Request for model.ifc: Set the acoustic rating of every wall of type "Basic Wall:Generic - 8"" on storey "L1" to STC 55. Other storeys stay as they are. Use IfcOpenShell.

First a look at what the model holds.

```python
import ifcopenshell
import ifcopenshell.util.element

model = ifcopenshell.open("model.ifc")
print(model.schema)
storey = next(s for s in model.by_type("IfcBuildingStorey") if s.Name == "L1")
walls = [e for e in ifcopenshell.util.element.get_decomposition(storey) if e.is_a("IfcWall")]
seen = {}
for e in walls:
    element_type = ifcopenshell.util.element.get_type(e)
    key = (element_type.Name if element_type != e and element_type else None, ifcopenshell.util.element.get_pset(e, "Pset_WallCommon", "AcousticRating"))
    seen[key] = seen.get(key, 0) + 1
for (name, value), count in sorted(seen.items(), key=str):
    print(count, "x", name, "|", value)
```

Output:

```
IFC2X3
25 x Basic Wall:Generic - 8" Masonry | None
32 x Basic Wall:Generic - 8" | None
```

```python
import ifcopenshell
import ifcopenshell.api.pset
import ifcopenshell.util.element

model = ifcopenshell.open("model.ifc")

storey = next(s for s in model.by_type("IfcBuildingStorey") if s.Name == "L1")
walls = [e for e in ifcopenshell.util.element.get_decomposition(storey) if e.is_a("IfcWall")]

count = 0
for e in walls:
    element_type = ifcopenshell.util.element.get_type(e)
    if element_type in (None, e) or element_type.Name != 'Basic Wall:Generic - 8"':
        continue
    # add_pset returns the element's existing set when there is one.
    pset = ifcopenshell.api.pset.add_pset(model, product=e, name="Pset_WallCommon")
    ifcopenshell.api.pset.edit_pset(model, pset=pset, properties={"AcousticRating": "STC 55"})
    count += 1

print(count, "walls updated")

model.write("model_v2.ifc")
```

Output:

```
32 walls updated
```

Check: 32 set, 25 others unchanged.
